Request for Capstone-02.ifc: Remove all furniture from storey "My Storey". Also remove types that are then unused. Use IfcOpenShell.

First a look at what the model holds.

```python
import ifcopenshell
import ifcopenshell.util.element

model = ifcopenshell.open("Capstone-02.ifc")
print(model.schema)
storey = next(s for s in model.by_type("IfcBuildingStorey") if s.Name == "My Storey")
furniture = [e for e in ifcopenshell.util.element.get_decomposition(storey) if e.is_a("IfcFurnishingElement")]
seen = {}
for e in furniture:
    element_type = ifcopenshell.util.element.get_type(e)
    name = element_type.Name if element_type not in (None, e) else None
    seen[name] = seen.get(name, 0) + 1
for name, count in sorted(seen.items(), key=str):
    print(count, "x", name)
```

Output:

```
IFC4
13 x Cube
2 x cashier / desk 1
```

```python
import ifcopenshell
import ifcopenshell.api.root
import ifcopenshell.util.element

model = ifcopenshell.open("Capstone-02.ifc")

storey = next(s for s in model.by_type("IfcBuildingStorey") if s.Name == "My Storey")
furniture = [e for e in ifcopenshell.util.element.get_decomposition(storey) if e.is_a("IfcFurnishingElement")]
types = {ifcopenshell.util.element.get_type(e) for e in furniture} - {None, *furniture}

for e in furniture:
    ifcopenshell.api.root.remove_product(model, product=e)
print(len(furniture), "removed")

unused = [t for t in types if not ifcopenshell.util.element.get_types(t)]
for t in unused:
    ifcopenshell.api.root.remove_product(model, product=t)
print(len(unused), "unused types removed")

model.write("Capstone-02_updated.ifc")
```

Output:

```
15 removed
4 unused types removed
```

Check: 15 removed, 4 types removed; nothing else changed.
